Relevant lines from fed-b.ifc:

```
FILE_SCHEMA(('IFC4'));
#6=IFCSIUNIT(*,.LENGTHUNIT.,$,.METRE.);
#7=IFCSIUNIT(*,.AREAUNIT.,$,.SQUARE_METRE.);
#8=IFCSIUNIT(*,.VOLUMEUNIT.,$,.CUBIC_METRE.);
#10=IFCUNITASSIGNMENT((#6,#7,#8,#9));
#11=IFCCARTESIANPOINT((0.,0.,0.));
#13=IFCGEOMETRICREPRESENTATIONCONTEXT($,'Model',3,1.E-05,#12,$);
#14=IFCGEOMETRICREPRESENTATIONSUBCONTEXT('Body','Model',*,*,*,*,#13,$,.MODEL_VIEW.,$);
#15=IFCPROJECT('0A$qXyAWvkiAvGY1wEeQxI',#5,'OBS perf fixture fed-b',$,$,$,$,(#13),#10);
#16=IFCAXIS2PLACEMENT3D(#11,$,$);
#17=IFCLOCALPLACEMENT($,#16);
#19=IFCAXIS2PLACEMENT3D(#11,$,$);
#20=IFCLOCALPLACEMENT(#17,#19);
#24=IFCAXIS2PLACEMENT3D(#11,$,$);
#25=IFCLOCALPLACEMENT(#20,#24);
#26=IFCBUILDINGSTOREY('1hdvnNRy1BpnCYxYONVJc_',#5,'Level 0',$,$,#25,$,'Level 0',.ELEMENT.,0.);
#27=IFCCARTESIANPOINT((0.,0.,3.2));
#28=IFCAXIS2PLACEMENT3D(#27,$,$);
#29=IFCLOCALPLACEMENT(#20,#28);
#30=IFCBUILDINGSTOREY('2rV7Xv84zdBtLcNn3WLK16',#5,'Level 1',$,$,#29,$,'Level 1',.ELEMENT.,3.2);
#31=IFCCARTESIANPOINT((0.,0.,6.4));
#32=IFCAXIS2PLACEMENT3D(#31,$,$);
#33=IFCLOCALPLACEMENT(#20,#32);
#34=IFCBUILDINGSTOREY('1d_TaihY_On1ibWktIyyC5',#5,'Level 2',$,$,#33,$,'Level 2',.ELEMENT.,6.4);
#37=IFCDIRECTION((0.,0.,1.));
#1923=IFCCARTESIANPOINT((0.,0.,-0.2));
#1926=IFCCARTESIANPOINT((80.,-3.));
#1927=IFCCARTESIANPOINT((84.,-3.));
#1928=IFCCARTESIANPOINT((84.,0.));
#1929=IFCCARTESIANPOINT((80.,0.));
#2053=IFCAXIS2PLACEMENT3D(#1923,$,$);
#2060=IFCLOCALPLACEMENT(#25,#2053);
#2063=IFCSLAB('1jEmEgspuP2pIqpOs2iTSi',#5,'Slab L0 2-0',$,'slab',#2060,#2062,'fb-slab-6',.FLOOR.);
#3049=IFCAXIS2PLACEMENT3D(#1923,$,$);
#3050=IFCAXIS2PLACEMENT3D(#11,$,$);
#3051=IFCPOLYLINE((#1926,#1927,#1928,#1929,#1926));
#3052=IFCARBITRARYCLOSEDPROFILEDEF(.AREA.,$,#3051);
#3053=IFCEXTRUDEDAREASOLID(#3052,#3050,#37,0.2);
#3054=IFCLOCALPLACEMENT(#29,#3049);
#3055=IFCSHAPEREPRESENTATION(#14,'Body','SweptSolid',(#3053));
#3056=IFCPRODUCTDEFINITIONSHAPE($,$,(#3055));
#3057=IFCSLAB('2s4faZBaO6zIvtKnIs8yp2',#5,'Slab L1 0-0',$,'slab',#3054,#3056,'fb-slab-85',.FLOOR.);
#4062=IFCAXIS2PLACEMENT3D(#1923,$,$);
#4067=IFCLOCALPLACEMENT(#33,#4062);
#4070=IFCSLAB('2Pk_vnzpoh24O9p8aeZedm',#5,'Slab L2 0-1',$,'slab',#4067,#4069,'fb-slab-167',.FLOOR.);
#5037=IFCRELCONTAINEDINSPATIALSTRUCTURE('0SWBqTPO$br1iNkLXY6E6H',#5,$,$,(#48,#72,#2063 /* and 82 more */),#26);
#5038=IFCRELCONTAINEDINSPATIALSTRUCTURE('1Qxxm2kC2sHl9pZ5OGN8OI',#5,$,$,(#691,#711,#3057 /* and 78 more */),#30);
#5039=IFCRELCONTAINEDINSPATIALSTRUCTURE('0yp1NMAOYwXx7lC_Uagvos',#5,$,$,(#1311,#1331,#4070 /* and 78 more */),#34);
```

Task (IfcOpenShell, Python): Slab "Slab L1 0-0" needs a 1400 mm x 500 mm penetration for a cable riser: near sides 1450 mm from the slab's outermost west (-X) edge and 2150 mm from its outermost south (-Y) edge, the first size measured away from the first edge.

```python
import numpy as np
import ifcopenshell
import ifcopenshell.api.feature
import ifcopenshell.api.geometry
import ifcopenshell.api.root
import ifcopenshell.geom
import ifcopenshell.util.placement
import ifcopenshell.util.representation
import ifcopenshell.util.shape
import ifcopenshell.util.unit

model = ifcopenshell.open("fed-b.ifc")
unit_scale = ifcopenshell.util.unit.calculate_unit_scale(model)
settings = ifcopenshell.geom.settings()


def volume(element):
    """Net volume in cubic metres, openings subtracted."""
    shape = ifcopenshell.geom.create_shape(settings, element)
    return ifcopenshell.util.shape.get_volume(shape.geometry)


slab = model.by_guid("2s4faZBaO6zIvtKnIs8yp2")
before = volume(slab)

# Extent in the slab's own axes, in metres. The edges named are its -X and -Y sides.
slab_shape = ifcopenshell.geom.create_shape(settings, slab)
vertices = ifcopenshell.util.shape.get_vertices(slab_shape.geometry)
x_min, y_min, bottom = vertices.min(axis=0)
top = vertices[:, 2].max()

opening = ifcopenshell.api.root.create_entity(model, ifc_class="IfcOpeningElement", name="Cable riser opening", predefined_type="OPENING")
context = ifcopenshell.util.representation.get_context(model, "Model", "Body", "MODEL_VIEW")
width, depth = 1.4, 0.5
outline = [(0.0, 0.0), (width, 0.0), (width, depth), (0.0, depth), (0.0, 0.0)]
# Overshoot both faces by 50 mm so the cut is clean.
shape = ifcopenshell.api.geometry.add_slab_representation(
    model, context=context, depth=top - bottom + 0.1, polyline=outline
)
ifcopenshell.api.geometry.assign_representation(model, product=opening, representation=shape)

matrix = ifcopenshell.util.placement.get_local_placement(slab.ObjectPlacement)
matrix[:, 3] = matrix @ np.append(np.array([x_min + 1.45, y_min + 2.15, bottom - 0.05]) / unit_scale, 1.0)
ifcopenshell.api.geometry.edit_object_placement(model, product=opening, matrix=matrix, is_si=False)
ifcopenshell.api.feature.add_feature(model, feature=opening, element=slab)

after = volume(slab)

print(f"slab volume {before:.3f} -> {after:.3f} m3")

model.write("fed-b_rev.ifc")
```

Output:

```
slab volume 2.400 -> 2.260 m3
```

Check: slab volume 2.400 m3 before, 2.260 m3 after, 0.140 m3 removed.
